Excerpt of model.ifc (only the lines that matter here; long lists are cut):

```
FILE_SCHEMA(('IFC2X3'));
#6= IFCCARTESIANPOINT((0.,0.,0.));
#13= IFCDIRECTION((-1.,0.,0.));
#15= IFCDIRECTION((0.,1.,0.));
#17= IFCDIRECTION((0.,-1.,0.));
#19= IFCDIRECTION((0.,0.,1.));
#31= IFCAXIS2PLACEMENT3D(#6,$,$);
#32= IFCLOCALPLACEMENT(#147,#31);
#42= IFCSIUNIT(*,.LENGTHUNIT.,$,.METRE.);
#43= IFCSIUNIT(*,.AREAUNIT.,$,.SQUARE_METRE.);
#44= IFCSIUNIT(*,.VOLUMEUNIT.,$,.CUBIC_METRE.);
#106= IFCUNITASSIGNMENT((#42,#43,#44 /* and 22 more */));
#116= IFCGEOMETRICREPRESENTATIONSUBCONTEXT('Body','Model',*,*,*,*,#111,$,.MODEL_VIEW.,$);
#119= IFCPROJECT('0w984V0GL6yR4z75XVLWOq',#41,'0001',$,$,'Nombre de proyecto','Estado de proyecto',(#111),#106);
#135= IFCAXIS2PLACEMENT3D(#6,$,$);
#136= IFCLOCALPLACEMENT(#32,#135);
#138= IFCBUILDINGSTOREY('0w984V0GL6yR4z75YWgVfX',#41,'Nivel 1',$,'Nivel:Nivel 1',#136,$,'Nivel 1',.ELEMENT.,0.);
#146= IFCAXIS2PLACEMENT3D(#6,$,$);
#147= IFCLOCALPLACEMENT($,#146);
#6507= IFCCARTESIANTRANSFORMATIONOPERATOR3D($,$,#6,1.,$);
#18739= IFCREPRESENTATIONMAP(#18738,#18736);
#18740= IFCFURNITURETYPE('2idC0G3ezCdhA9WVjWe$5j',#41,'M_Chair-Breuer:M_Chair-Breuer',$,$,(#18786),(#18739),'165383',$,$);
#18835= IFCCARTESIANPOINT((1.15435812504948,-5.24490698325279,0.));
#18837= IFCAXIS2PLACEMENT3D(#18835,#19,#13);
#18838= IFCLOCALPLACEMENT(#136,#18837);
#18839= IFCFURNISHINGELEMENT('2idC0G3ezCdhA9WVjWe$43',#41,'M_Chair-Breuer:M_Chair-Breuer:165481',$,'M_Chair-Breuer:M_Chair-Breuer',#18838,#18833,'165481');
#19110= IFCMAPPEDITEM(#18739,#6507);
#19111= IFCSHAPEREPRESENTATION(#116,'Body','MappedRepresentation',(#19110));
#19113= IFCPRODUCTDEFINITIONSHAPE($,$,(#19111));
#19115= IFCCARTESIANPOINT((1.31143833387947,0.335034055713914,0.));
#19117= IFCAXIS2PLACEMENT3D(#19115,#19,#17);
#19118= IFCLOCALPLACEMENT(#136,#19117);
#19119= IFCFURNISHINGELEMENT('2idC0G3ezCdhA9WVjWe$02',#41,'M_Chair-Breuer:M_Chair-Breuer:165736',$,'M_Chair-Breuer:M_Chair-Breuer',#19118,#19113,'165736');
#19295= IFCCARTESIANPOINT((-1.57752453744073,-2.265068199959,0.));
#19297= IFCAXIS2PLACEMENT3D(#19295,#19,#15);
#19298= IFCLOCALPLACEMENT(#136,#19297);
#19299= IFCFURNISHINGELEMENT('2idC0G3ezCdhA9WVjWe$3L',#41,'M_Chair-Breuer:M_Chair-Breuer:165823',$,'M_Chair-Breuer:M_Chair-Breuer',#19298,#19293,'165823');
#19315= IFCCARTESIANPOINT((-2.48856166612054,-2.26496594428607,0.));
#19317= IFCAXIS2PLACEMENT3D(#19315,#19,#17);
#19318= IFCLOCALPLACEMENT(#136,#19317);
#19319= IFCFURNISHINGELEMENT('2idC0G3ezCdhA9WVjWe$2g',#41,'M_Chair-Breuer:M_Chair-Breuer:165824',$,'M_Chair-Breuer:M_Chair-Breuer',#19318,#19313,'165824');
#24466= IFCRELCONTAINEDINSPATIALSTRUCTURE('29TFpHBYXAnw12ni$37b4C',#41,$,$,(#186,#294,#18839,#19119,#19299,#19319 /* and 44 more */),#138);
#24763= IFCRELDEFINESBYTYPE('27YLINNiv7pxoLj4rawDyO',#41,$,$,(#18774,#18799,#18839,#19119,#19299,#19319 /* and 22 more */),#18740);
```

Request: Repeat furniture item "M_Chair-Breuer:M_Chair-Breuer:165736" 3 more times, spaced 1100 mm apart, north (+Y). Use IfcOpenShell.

```python
import numpy as np
import ifcopenshell
import ifcopenshell.api.geometry
import ifcopenshell.api.root
import ifcopenshell.util.element
import ifcopenshell.util.placement
import ifcopenshell.util.unit

model = ifcopenshell.open("model.ifc")
unit_scale = ifcopenshell.util.unit.calculate_unit_scale(model)


def reuse_history(source, copy):
    """copy_class also copies each property set's owner history, people and application; keep the originals."""
    for rel in copy.IsDefinedBy:
        if rel.is_a("IfcRelDefinesByProperties") and (history := rel.RelatingPropertyDefinition.OwnerHistory):
            rel.RelatingPropertyDefinition.OwnerHistory = source.OwnerHistory
            ifcopenshell.util.element.remove_deep2(model, history)


source = model.by_guid("2idC0G3ezCdhA9WVjWe$02")
base = ifcopenshell.util.placement.get_local_placement(source.ObjectPlacement)
step = np.array([0.0, 1.0, 0.0]) * 1.1 / unit_scale

for i in range(1, 4):
    copy = ifcopenshell.api.root.copy_class(model, product=source)
    copy.Representation = ifcopenshell.util.element.copy_deep(
        model, source.Representation, exclude=["IfcGeometricRepresentationContext", "IfcRepresentationMap"]
    )
    copy.Name = "M_Chair-Breuer:M_Chair-Breuer"
    copy.Tag = None
    reuse_history(source, copy)
    matrix = base.copy()
    matrix[:3, 3] += i * step
    print("added at", matrix[:3, 3].round(3) + 0.0)
    ifcopenshell.api.geometry.edit_object_placement(model, product=copy, matrix=matrix, is_si=False)

model.write("model-out.ifc")
```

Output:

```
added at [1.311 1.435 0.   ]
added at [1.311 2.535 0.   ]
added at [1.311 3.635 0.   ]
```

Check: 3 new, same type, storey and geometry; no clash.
